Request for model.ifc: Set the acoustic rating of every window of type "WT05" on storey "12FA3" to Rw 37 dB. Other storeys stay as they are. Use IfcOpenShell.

First a look at what the model holds.

```python
import ifcopenshell
import ifcopenshell.util.element

model = ifcopenshell.open("model.ifc")
print(model.schema)
storey = next(s for s in model.by_type("IfcBuildingStorey") if s.Name == "12FA3")
windows = [e for e in ifcopenshell.util.element.get_decomposition(storey) if e.is_a("IfcWindow")]
seen = {}
for e in windows:
    element_type = ifcopenshell.util.element.get_type(e)
    key = (element_type.Name if element_type != e and element_type else None, ifcopenshell.util.element.get_pset(e, "Pset_WindowCommon", "AcousticRating"))
    seen[key] = seen.get(key, 0) + 1
for (name, value), count in sorted(seen.items(), key=str):
    print(count, "x", name, "|", value)
```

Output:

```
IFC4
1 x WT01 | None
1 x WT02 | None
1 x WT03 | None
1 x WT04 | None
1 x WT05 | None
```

```python
import ifcopenshell
import ifcopenshell.api.pset
import ifcopenshell.util.element

model = ifcopenshell.open("model.ifc")

storey = next(s for s in model.by_type("IfcBuildingStorey") if s.Name == "12FA3")
windows = [e for e in ifcopenshell.util.element.get_decomposition(storey) if e.is_a("IfcWindow")]

count = 0
for e in windows:
    element_type = ifcopenshell.util.element.get_type(e)
    if element_type in (None, e) or element_type.Name != "WT05":
        continue
    # add_pset returns the element's existing set when there is one.
    pset = ifcopenshell.api.pset.add_pset(model, product=e, name="Pset_WindowCommon")
    ifcopenshell.api.pset.edit_pset(model, pset=pset, properties={"AcousticRating": "Rw 37 dB"})
    count += 1

print(count, "windows updated")

model.write("model_updated.ifc")
```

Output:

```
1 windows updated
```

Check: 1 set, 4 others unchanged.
